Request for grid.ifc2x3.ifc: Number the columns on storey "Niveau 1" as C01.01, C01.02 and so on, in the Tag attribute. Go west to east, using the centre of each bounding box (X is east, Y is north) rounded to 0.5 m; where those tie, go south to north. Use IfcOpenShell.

First a look at what the model holds.

```python
import ifcopenshell
import ifcopenshell.util.element
import ifcopenshell.util.placement

model = ifcopenshell.open("grid.ifc2x3.ifc")
print(model.schema)
storey = next(s for s in model.by_type("IfcBuildingStorey") if s.Name == "Niveau 1")
columns = [e for e in ifcopenshell.util.element.get_decomposition(storey) if e.is_a("IfcColumn")]
for e in sorted(columns, key=lambda e: e.id()):
    origin = ifcopenshell.util.placement.get_local_placement(e.ObjectPlacement)[:3, 3]
    print(e.id(), e.Tag, e.Name, origin.round(2) + 0.0, sep=" | ")
```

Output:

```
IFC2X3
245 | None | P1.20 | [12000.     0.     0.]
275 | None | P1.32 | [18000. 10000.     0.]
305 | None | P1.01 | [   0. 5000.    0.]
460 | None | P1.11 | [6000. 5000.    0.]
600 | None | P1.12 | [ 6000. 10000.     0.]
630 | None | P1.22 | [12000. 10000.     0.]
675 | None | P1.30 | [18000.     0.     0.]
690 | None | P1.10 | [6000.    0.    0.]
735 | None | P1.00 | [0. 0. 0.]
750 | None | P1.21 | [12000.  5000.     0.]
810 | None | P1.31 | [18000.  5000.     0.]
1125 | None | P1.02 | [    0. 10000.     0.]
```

```python
import ifcopenshell
import ifcopenshell.geom
import ifcopenshell.util.element
import ifcopenshell.util.shape

model = ifcopenshell.open("grid.ifc2x3.ifc")
settings = ifcopenshell.geom.settings()
settings.set("use-world-coords", True)


def centre(element):
    shape = ifcopenshell.geom.create_shape(settings, element)
    return ifcopenshell.util.shape.get_bbox_centroid(shape.geometry)


storey = next(s for s in model.by_type("IfcBuildingStorey") if s.Name == "Niveau 1")
columns = [e for e in ifcopenshell.util.element.get_decomposition(storey) if e.is_a("IfcColumn")]

# Insertion points can sit at a corner or the storey origin, so sort by the geometry (in metres).
centres = {e: centre(e) for e in columns}
columns.sort(key=lambda e: (round(centres[e][0] / 0.5), centres[e][1]))

for i, e in enumerate(columns, start=1):
    number = f"C01.{i:02d}"
    e.Tag = number
    print(e.id(), number)

model.write("grid.ifc2x3_edited.ifc")
```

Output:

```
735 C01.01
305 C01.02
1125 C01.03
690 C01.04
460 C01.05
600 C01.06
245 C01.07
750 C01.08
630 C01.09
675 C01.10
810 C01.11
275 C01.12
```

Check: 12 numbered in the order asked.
